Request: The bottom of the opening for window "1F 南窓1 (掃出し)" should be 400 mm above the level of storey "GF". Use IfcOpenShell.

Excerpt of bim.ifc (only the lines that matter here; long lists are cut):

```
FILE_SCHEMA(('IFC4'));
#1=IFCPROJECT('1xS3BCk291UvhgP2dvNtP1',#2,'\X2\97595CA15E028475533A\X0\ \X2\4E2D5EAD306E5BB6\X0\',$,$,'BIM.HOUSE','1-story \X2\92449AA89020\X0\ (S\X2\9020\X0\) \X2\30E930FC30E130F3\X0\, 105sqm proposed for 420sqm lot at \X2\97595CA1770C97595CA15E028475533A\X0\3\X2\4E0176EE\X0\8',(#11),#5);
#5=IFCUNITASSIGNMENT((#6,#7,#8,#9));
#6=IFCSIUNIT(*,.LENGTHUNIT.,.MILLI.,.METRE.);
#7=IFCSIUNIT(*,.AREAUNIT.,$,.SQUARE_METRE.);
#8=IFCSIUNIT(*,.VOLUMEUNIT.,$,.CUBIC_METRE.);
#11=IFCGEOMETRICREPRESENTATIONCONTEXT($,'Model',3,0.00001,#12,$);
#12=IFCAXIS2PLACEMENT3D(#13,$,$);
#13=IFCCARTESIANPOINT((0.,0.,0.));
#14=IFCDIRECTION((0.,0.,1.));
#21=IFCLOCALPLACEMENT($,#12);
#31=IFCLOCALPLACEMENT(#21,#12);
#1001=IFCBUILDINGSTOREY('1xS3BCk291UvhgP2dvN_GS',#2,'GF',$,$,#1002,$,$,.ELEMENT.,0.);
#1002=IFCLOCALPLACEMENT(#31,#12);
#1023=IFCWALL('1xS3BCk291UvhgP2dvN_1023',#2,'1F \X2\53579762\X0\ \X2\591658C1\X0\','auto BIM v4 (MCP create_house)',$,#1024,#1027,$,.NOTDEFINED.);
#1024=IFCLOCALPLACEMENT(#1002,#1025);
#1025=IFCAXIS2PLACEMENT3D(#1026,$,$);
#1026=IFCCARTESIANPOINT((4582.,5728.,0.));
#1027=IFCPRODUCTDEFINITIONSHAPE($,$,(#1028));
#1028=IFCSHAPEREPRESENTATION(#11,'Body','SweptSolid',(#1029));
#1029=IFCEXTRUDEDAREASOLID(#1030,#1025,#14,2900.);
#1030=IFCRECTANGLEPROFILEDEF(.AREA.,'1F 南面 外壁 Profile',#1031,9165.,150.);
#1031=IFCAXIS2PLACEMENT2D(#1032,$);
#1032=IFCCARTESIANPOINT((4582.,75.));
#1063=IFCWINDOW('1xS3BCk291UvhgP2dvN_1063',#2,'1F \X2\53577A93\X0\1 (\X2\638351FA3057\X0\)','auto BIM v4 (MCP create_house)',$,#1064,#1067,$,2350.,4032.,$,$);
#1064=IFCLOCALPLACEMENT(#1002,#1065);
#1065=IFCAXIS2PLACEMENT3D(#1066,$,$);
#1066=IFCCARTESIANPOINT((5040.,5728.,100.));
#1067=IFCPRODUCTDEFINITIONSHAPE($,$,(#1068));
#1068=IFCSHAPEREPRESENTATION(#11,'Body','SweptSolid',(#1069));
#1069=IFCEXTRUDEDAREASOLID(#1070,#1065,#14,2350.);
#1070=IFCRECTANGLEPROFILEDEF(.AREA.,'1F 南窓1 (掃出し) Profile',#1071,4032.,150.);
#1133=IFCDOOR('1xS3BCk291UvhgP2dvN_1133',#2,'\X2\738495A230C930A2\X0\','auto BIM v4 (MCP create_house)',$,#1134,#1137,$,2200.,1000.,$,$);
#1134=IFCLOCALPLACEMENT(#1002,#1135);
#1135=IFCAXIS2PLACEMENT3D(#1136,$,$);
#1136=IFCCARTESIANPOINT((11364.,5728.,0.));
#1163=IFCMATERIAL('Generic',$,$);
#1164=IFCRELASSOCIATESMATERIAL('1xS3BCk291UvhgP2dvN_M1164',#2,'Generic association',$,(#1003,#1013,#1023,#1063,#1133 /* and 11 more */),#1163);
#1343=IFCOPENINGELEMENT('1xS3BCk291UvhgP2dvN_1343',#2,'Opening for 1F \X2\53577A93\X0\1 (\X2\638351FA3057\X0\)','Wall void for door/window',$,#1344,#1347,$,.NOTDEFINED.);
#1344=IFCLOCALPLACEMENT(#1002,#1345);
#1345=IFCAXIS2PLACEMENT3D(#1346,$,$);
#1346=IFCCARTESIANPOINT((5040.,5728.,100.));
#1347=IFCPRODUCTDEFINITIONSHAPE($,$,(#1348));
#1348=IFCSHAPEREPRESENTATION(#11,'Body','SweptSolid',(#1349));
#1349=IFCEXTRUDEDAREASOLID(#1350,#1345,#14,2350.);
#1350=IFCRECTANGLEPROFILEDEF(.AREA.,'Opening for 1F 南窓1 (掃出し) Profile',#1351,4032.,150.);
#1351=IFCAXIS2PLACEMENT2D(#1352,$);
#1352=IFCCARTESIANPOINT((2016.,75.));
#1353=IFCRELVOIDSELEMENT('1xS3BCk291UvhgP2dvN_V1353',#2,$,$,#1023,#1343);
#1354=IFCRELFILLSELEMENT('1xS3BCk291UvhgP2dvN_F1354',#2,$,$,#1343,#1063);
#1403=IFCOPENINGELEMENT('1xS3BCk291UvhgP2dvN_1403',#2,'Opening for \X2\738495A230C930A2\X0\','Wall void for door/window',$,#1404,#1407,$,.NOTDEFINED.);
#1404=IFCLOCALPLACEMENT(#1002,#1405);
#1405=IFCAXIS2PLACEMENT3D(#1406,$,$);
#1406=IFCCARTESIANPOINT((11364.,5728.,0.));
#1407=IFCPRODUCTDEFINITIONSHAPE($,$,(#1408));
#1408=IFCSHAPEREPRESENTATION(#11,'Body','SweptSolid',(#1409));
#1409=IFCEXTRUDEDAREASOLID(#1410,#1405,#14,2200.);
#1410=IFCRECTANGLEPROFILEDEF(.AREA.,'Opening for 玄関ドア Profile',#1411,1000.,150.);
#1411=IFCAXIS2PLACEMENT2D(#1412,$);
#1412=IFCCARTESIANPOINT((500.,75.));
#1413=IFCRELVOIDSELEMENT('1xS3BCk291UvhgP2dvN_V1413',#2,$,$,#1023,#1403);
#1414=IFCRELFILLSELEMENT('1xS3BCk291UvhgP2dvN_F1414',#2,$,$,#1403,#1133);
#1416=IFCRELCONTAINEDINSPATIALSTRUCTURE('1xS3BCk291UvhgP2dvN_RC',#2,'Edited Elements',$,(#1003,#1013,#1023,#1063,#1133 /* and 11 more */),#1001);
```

```python
import numpy as np
import ifcopenshell
import ifcopenshell.api.geometry
import ifcopenshell.geom
import ifcopenshell.util.element
import ifcopenshell.util.placement
import ifcopenshell.util.shape
import ifcopenshell.util.unit

model = ifcopenshell.open("bim.ifc")
unit_scale = ifcopenshell.util.unit.calculate_unit_scale(model)

window = model.by_id(1063)
opening = window.FillsVoids[0].RelatingOpeningElement
storey = ifcopenshell.util.element.get_container(window, ifc_class="IfcBuildingStorey")
level = ifcopenshell.util.placement.get_local_placement(storey.ObjectPlacement)[2, 3]

# The opening's origin need not be at the sill, so measure its lowest point.
shape = ifcopenshell.geom.create_shape(ifcopenshell.geom.settings(), opening)
bottom = ifcopenshell.util.shape.get_shape_bottom_elevation(shape, shape.geometry) / unit_scale
dz = level + 0.4 / unit_scale - bottom

shift = np.array([0.0, 0.0, dz])
# The window is not placed relative to its opening, so move both.
for product in (opening, window):
    matrix = ifcopenshell.util.placement.get_local_placement(product.ObjectPlacement)
    matrix[:3, 3] += shift
    ifcopenshell.api.geometry.edit_object_placement(model, product=product, matrix=matrix, is_si=False)

print(f"moved by {dz * unit_scale:+.3f} m")

model.write("bim-out.ifc")
```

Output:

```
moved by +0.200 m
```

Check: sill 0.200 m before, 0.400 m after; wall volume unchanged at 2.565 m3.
